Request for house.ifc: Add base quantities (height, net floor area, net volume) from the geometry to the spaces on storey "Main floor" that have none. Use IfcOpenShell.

First a look at what the model holds.

```python
import ifcopenshell
import ifcopenshell.util.element
import ifcopenshell.util.unit

model = ifcopenshell.open("house.ifc")
print(model.schema)
for unit_type in ("LENGTHUNIT", "AREAUNIT", "VOLUMEUNIT"):
    print(unit_type, ifcopenshell.util.unit.calculate_unit_scale(model, unit_type))
storey = next(s for s in model.by_type("IfcBuildingStorey") if s.Name == "Main floor")
spaces = [e for e in ifcopenshell.util.element.get_decomposition(storey) if e.is_a("IfcSpace")]
for e in sorted(spaces, key=lambda e: e.id()):
    print(e.id(), e.is_a(), e.Name, list(ifcopenshell.util.element.get_psets(e, qtos_only=True)), sep=" | ")
```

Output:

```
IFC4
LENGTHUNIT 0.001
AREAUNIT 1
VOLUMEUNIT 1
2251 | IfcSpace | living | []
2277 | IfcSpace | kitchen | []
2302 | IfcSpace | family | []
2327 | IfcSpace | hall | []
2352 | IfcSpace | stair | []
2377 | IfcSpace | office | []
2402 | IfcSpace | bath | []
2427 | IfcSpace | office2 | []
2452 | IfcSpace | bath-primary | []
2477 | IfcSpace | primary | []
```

```python
import ifcopenshell
import ifcopenshell.api.pset
import ifcopenshell.geom
import ifcopenshell.util.element
import ifcopenshell.util.shape
import ifcopenshell.util.unit

model = ifcopenshell.open("house.ifc")
unit_scale = ifcopenshell.util.unit.calculate_unit_scale(model)
area_scale = ifcopenshell.util.unit.calculate_unit_scale(model, "AREAUNIT")
volume_scale = ifcopenshell.util.unit.calculate_unit_scale(model, "VOLUMEUNIT")
settings = ifcopenshell.geom.settings()

storey = next(s for s in model.by_type("IfcBuildingStorey") if s.Name == "Main floor")
spaces = [e for e in ifcopenshell.util.element.get_decomposition(storey) if e.is_a("IfcSpace")]

for e in sorted(spaces, key=lambda e: e.id()):
    if ifcopenshell.util.element.get_psets(e, qtos_only=True, should_inherit=False):
        continue
    # Geometry comes back in metres, in the element's own axes.
    shape = ifcopenshell.geom.create_shape(settings, e)
    values = {
        "Height": ifcopenshell.util.shape.get_z(shape.geometry) / unit_scale,
        "NetFloorArea": ifcopenshell.util.shape.get_footprint_area(shape.geometry) / area_scale,
        "NetVolume": ifcopenshell.util.shape.get_volume(shape.geometry) / volume_scale,
    }
    qto = ifcopenshell.api.pset.add_qto(model, product=e, name="Qto_SpaceBaseQuantities")
    ifcopenshell.api.pset.edit_qto(model, qto=qto, properties=values)
    print(e.id(), {k: round(v, 3) for k, v in values.items()})

model.write("house-out.ifc")
```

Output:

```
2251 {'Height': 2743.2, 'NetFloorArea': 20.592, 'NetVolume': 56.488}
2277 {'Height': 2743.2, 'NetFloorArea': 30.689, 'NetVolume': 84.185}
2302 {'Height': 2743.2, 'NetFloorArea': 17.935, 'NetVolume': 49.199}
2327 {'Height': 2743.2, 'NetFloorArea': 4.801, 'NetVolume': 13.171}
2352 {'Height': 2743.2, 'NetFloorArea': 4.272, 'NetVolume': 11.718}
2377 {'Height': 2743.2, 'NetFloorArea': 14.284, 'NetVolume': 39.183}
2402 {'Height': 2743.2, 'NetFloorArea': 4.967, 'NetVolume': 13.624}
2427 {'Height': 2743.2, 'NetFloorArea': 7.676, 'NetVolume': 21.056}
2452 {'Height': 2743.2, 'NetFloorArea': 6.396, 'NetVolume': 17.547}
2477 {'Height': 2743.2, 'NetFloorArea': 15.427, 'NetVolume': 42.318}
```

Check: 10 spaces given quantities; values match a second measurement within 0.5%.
